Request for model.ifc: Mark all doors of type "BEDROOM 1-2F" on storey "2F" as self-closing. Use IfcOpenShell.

First a look at what the model holds.

```python
import ifcopenshell
import ifcopenshell.util.element

model = ifcopenshell.open("model.ifc")
print(model.schema)
storey = next(s for s in model.by_type("IfcBuildingStorey") if s.Name == "2F")
doors = [e for e in ifcopenshell.util.element.get_decomposition(storey) if e.is_a("IfcDoor")]
seen = {}
for e in doors:
    element_type = ifcopenshell.util.element.get_type(e)
    key = (element_type.Name if element_type != e and element_type else None, ifcopenshell.util.element.get_pset(e, "Pset_DoorCommon", "SelfClosing"))
    seen[key] = seen.get(key, 0) + 1
for (name, value), count in sorted(seen.items(), key=str):
    print(count, "x", name, "|", value)
```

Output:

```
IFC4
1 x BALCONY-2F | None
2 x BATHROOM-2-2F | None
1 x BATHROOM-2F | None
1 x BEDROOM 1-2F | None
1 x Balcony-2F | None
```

```python
import ifcopenshell
import ifcopenshell.api.pset
import ifcopenshell.util.element

model = ifcopenshell.open("model.ifc")

storey = next(s for s in model.by_type("IfcBuildingStorey") if s.Name == "2F")
doors = [e for e in ifcopenshell.util.element.get_decomposition(storey) if e.is_a("IfcDoor")]

count = 0
for e in doors:
    element_type = ifcopenshell.util.element.get_type(e)
    if element_type in (None, e) or element_type.Name != "BEDROOM 1-2F":
        continue
    # add_pset returns the element's existing set when there is one.
    pset = ifcopenshell.api.pset.add_pset(model, product=e, name="Pset_DoorCommon")
    ifcopenshell.api.pset.edit_pset(model, pset=pset, properties={"SelfClosing": True})
    count += 1

print(count, "doors updated")

model.write("model-out.ifc")
```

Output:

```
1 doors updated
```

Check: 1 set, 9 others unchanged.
